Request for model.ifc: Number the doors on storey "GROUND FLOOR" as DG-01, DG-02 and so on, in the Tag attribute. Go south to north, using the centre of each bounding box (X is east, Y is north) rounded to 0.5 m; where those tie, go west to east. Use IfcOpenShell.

First a look at what the model holds.

```python
import ifcopenshell
import ifcopenshell.util.element
import ifcopenshell.util.placement

model = ifcopenshell.open("model.ifc")
print(model.schema)
storey = next(s for s in model.by_type("IfcBuildingStorey") if s.Name == "GROUND FLOOR")
doors = [e for e in ifcopenshell.util.element.get_decomposition(storey) if e.is_a("IfcDoor")]
for e in sorted(doors, key=lambda e: e.id()):
    origin = ifcopenshell.util.placement.get_local_placement(e.ObjectPlacement)[:3, 3]
    print(e.id(), e.Tag, e.Name, origin.round(2) + 0.0, sep=" | ")
```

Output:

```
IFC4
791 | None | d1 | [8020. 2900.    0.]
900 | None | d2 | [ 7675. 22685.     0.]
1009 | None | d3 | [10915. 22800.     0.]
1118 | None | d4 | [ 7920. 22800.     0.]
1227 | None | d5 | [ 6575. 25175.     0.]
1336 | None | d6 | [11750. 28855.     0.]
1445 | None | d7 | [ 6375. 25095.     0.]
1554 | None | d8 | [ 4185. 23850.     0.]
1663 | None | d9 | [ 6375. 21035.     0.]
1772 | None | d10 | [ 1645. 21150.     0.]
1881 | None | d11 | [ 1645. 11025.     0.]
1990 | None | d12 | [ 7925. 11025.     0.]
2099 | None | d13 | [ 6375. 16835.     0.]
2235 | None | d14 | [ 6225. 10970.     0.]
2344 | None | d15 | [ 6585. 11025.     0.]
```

```python
import ifcopenshell
import ifcopenshell.geom
import ifcopenshell.util.element
import ifcopenshell.util.shape

model = ifcopenshell.open("model.ifc")
settings = ifcopenshell.geom.settings()
settings.set("use-world-coords", True)


def centre(element):
    shape = ifcopenshell.geom.create_shape(settings, element)
    return ifcopenshell.util.shape.get_bbox_centroid(shape.geometry)


storey = next(s for s in model.by_type("IfcBuildingStorey") if s.Name == "GROUND FLOOR")
doors = [e for e in ifcopenshell.util.element.get_decomposition(storey) if e.is_a("IfcDoor")]

# Insertion points can sit at a corner or the storey origin, so sort by the geometry (in metres).
centres = {e: centre(e) for e in doors}
doors.sort(key=lambda e: (round(centres[e][1] / 0.5), centres[e][0]))

for i, e in enumerate(doors, start=1):
    number = f"DG-{i:02d}"
    e.Tag = number
    print(e.id(), number)

model.write("model_edited.ifc")
```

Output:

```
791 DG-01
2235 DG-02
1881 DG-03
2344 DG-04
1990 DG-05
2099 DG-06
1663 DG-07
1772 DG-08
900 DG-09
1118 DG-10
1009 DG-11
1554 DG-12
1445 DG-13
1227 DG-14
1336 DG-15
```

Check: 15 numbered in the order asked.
